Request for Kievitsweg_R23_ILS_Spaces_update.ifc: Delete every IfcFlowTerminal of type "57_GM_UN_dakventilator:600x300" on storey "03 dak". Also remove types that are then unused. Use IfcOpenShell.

First a look at what the model holds.

```python
import ifcopenshell
import ifcopenshell.util.element

model = ifcopenshell.open("Kievitsweg_R23_ILS_Spaces_update.ifc")
print(model.schema)
storey = next(s for s in model.by_type("IfcBuildingStorey") if s.Name == "03 dak")
terminals = [e for e in ifcopenshell.util.element.get_decomposition(storey) if e.is_a("IfcFlowTerminal")]
seen = {}
for e in terminals:
    element_type = ifcopenshell.util.element.get_type(e)
    name = element_type.Name if element_type not in (None, e) else None
    seen[name] = seen.get(name, 0) + 1
for name, count in sorted(seen.items(), key=str):
    print(count, "x", name)
```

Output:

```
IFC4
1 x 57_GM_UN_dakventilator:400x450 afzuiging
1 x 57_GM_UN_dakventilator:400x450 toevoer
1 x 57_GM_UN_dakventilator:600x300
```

```python
import ifcopenshell
import ifcopenshell.api.root
import ifcopenshell.util.element

model = ifcopenshell.open("Kievitsweg_R23_ILS_Spaces_update.ifc")

storey = next(s for s in model.by_type("IfcBuildingStorey") if s.Name == "03 dak")
terminals = [e for e in ifcopenshell.util.element.get_decomposition(storey) if e.is_a("IfcFlowTerminal")]
targets = [e for e in terminals if (t := ifcopenshell.util.element.get_type(e)) not in (None, e) and t.Name == "57_GM_UN_dakventilator:600x300"]
types = {ifcopenshell.util.element.get_type(e) for e in targets} - {None, *targets}

for e in targets:
    ifcopenshell.api.root.remove_product(model, product=e)
print(len(targets), "removed")

unused = [t for t in types if not ifcopenshell.util.element.get_types(t)]
for t in unused:
    ifcopenshell.api.root.remove_product(model, product=t)
print(len(unused), "unused types removed")

model.write("Kievitsweg_R23_ILS_Spaces_update-out.ifc")
```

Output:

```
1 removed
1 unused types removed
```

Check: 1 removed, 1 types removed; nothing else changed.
